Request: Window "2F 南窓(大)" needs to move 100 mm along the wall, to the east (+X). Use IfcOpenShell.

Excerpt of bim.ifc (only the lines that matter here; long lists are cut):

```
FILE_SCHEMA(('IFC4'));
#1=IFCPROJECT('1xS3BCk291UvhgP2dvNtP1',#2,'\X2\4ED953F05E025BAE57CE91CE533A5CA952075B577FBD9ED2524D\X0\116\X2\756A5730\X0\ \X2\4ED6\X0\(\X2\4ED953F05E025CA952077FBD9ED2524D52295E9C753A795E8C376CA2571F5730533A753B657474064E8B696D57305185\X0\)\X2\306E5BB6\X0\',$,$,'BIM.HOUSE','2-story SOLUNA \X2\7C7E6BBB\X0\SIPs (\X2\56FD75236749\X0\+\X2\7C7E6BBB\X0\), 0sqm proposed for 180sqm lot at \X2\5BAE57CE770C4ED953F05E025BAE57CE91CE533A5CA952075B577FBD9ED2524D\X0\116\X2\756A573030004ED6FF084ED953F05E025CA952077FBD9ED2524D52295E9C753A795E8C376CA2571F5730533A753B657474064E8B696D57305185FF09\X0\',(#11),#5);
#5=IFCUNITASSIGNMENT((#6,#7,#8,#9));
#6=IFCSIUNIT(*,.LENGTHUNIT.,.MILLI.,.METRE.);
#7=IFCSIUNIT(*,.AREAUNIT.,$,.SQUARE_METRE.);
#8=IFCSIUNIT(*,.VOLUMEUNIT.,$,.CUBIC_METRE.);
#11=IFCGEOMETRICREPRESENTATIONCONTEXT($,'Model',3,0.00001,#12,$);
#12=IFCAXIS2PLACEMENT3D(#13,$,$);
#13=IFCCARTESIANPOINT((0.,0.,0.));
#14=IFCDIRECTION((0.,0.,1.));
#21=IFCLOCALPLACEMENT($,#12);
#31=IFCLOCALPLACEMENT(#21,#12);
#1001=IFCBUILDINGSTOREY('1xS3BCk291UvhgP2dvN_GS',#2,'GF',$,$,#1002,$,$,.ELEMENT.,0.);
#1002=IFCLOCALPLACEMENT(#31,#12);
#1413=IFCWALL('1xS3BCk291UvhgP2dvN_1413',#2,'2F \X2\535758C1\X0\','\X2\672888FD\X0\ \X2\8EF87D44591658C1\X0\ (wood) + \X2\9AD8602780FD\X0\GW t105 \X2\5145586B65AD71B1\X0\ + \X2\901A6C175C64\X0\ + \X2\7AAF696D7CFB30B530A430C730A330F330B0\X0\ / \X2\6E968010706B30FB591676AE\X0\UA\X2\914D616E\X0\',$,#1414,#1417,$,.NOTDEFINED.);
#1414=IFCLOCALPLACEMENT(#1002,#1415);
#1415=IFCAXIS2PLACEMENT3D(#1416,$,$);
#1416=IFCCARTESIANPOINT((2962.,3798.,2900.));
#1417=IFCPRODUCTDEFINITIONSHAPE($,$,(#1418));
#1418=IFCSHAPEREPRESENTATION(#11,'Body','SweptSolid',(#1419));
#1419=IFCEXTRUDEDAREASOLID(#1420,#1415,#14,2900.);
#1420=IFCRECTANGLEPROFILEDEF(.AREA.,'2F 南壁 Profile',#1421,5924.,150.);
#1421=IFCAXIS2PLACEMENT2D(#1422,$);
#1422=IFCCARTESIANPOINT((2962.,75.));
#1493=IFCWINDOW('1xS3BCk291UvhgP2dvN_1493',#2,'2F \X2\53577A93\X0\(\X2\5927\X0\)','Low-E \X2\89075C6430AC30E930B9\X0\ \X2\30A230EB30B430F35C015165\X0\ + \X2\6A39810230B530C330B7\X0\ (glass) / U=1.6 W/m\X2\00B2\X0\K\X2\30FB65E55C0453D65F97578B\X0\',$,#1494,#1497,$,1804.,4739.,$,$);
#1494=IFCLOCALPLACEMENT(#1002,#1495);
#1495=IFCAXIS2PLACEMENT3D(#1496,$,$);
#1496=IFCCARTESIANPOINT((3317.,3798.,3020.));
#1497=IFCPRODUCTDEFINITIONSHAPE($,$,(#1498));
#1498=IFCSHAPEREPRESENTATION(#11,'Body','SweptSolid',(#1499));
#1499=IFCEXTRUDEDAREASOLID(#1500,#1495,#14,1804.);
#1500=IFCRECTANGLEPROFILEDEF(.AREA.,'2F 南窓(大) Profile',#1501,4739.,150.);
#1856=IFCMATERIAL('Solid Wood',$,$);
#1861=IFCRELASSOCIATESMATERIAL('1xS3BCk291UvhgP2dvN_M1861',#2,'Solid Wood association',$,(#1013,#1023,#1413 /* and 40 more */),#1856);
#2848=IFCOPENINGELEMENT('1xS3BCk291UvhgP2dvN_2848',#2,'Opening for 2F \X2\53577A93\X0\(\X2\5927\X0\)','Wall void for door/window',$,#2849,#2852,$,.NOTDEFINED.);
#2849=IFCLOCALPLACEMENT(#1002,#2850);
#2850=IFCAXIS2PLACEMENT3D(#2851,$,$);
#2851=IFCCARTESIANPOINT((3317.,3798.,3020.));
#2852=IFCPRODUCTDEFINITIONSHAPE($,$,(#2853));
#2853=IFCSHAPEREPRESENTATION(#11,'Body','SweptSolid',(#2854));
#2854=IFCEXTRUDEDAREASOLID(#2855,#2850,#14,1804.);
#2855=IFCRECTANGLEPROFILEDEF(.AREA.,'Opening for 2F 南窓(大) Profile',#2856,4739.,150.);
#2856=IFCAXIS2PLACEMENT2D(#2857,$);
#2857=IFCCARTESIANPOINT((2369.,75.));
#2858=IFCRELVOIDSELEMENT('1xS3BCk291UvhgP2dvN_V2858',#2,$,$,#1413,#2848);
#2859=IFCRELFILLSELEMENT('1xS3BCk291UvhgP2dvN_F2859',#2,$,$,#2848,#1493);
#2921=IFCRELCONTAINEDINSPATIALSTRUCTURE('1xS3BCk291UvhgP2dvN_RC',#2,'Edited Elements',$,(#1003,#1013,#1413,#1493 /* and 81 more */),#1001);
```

```python
import ifcopenshell
import ifcopenshell.api.geometry
import ifcopenshell.util.placement
import ifcopenshell.util.unit

model = ifcopenshell.open("bim.ifc")
unit_scale = ifcopenshell.util.unit.calculate_unit_scale(model)

window = model.by_id(1493)
opening = window.FillsVoids[0].RelatingOpeningElement
wall = opening.VoidsElements[0].RelatingBuildingElement

wall_matrix = ifcopenshell.util.placement.get_local_placement(wall.ObjectPlacement)
shift = wall_matrix[:3, 0] * 0.1 / unit_scale
before = ifcopenshell.util.placement.get_local_placement(window.ObjectPlacement)[:3, 3].copy()

# The window is not placed relative to its opening, so move both.
for product in (opening, window):
    matrix = ifcopenshell.util.placement.get_local_placement(product.ObjectPlacement)
    matrix[:3, 3] += shift
    ifcopenshell.api.geometry.edit_object_placement(model, product=product, matrix=matrix, is_si=False)

after = ifcopenshell.util.placement.get_local_placement(window.ObjectPlacement)[:3, 3]
print("window moved by", (after - before).round(3) + 0.0)

model.write("bim_updated.ifc")
```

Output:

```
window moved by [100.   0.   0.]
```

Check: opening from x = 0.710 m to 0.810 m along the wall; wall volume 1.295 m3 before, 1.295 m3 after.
